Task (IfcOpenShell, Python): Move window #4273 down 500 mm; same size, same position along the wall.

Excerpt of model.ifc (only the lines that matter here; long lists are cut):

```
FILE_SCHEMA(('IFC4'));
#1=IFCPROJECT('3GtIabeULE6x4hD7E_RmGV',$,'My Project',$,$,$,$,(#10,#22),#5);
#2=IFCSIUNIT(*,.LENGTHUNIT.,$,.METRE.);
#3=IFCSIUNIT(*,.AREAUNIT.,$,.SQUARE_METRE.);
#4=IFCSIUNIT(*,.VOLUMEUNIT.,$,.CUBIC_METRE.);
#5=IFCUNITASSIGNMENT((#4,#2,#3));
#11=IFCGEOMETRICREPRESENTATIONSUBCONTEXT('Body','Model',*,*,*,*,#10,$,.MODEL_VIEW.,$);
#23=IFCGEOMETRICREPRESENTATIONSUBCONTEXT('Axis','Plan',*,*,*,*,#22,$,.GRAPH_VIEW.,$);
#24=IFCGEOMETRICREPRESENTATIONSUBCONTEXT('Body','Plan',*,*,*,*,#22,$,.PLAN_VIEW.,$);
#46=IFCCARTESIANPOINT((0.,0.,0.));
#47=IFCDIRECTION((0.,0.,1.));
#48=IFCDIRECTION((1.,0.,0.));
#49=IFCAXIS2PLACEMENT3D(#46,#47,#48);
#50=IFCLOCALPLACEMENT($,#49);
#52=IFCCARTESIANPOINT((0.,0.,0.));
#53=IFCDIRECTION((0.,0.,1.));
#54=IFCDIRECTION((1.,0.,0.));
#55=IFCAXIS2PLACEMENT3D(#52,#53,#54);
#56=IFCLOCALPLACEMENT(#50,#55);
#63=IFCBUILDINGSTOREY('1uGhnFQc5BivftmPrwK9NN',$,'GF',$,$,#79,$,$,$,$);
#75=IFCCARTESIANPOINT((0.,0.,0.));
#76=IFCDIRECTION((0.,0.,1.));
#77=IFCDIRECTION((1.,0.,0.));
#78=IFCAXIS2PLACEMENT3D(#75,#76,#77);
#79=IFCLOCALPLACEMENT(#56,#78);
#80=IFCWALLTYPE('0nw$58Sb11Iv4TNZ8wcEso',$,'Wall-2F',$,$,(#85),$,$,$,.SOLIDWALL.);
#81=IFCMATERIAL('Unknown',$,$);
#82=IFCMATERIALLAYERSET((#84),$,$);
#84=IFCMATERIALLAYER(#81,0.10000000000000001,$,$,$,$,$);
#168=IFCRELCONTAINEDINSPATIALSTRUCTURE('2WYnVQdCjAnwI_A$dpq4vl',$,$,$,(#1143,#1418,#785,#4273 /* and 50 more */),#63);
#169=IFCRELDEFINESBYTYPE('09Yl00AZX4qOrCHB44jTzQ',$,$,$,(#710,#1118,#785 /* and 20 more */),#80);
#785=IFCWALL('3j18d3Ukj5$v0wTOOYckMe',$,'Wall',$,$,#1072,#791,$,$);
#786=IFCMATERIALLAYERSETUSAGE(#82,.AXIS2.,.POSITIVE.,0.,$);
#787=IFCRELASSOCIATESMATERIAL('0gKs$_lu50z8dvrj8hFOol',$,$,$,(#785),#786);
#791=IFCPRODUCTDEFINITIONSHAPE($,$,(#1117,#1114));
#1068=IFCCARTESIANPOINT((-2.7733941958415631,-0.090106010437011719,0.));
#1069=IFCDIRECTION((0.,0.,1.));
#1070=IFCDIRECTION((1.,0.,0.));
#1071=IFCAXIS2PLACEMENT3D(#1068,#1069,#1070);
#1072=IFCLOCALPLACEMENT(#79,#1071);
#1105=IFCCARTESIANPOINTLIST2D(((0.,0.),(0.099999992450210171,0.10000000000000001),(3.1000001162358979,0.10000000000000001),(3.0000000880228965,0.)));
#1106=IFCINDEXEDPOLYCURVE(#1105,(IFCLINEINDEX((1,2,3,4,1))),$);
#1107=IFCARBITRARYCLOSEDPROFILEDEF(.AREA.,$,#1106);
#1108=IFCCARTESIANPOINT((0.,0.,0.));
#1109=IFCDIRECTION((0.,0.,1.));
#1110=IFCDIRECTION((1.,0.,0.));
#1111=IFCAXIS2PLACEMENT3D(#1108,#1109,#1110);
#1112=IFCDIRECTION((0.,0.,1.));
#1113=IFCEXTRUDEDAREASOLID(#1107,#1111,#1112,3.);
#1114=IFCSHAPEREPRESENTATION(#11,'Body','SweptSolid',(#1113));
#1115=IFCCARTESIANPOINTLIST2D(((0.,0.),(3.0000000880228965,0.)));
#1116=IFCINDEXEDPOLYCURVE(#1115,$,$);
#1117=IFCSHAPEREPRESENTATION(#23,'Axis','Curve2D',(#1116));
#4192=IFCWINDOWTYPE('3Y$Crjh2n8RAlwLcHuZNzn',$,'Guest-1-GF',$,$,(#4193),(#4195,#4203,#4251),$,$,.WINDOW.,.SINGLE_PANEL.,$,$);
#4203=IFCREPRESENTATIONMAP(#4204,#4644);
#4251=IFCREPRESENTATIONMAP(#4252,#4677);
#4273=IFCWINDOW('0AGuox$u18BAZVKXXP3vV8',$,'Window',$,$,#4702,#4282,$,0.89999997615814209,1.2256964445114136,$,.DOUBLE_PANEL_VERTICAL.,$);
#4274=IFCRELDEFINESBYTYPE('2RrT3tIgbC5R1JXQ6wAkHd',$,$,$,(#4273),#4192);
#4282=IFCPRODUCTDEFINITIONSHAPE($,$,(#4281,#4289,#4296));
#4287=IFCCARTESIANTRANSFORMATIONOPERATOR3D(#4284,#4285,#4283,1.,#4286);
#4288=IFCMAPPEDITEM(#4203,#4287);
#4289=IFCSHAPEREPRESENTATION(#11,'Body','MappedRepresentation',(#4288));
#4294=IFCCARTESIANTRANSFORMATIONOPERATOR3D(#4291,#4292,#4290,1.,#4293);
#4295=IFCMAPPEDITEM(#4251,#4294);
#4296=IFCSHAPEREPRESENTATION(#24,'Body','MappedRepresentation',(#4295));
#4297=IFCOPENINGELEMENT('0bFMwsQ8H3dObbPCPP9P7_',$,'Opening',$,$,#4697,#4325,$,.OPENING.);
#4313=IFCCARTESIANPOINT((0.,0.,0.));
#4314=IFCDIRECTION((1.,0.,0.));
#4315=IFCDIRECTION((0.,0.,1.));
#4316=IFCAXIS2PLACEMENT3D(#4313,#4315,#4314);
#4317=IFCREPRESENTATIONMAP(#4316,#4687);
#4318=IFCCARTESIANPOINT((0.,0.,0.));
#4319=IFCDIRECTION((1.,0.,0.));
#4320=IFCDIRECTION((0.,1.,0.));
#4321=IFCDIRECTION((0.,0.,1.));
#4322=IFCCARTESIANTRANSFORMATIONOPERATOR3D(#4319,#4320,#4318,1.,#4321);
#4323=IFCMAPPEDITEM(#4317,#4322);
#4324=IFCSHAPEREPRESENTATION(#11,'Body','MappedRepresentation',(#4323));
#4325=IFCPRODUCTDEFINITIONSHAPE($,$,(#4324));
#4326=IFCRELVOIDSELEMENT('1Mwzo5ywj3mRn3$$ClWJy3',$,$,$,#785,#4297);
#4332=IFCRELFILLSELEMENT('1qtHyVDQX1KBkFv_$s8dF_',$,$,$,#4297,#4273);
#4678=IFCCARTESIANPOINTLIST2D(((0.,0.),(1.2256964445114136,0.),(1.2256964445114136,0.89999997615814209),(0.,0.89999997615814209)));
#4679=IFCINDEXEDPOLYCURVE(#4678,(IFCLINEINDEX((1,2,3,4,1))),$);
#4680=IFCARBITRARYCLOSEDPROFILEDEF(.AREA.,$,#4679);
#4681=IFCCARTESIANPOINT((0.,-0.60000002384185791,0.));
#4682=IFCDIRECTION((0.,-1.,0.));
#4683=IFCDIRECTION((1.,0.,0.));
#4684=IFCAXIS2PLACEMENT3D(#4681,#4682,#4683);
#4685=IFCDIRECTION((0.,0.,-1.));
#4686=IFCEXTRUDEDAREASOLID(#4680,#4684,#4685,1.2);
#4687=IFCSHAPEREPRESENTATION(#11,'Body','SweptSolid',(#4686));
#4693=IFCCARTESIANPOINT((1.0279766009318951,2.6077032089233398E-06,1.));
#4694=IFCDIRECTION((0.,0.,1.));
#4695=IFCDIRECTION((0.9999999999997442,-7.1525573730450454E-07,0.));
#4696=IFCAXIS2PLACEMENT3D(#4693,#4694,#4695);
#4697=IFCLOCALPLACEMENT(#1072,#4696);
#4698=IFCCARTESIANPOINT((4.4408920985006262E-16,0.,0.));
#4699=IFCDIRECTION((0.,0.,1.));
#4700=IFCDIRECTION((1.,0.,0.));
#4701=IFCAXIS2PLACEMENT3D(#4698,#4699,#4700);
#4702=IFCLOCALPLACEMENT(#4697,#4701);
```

```python
import numpy as np
import ifcopenshell
import ifcopenshell.api.geometry
import ifcopenshell.util.placement
import ifcopenshell.util.unit

model = ifcopenshell.open("model.ifc")
unit_scale = ifcopenshell.util.unit.calculate_unit_scale(model)

window = model.by_guid("0AGuox$u18BAZVKXXP3vV8")
opening = window.FillsVoids[0].RelatingOpeningElement
dz = -0.5 / unit_scale

shift = np.array([0.0, 0.0, dz])
# The window is placed relative to its opening, so it follows when the opening moves.
matrix = ifcopenshell.util.placement.get_local_placement(opening.ObjectPlacement)
matrix[:3, 3] += shift
ifcopenshell.api.geometry.edit_object_placement(
    model, product=opening, matrix=matrix, is_si=False, should_transform_children=True
)

print(f"moved by {dz * unit_scale:+.3f} m")

model.write("model_updated.ifc")
```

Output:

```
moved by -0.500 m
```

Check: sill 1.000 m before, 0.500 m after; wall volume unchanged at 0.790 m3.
